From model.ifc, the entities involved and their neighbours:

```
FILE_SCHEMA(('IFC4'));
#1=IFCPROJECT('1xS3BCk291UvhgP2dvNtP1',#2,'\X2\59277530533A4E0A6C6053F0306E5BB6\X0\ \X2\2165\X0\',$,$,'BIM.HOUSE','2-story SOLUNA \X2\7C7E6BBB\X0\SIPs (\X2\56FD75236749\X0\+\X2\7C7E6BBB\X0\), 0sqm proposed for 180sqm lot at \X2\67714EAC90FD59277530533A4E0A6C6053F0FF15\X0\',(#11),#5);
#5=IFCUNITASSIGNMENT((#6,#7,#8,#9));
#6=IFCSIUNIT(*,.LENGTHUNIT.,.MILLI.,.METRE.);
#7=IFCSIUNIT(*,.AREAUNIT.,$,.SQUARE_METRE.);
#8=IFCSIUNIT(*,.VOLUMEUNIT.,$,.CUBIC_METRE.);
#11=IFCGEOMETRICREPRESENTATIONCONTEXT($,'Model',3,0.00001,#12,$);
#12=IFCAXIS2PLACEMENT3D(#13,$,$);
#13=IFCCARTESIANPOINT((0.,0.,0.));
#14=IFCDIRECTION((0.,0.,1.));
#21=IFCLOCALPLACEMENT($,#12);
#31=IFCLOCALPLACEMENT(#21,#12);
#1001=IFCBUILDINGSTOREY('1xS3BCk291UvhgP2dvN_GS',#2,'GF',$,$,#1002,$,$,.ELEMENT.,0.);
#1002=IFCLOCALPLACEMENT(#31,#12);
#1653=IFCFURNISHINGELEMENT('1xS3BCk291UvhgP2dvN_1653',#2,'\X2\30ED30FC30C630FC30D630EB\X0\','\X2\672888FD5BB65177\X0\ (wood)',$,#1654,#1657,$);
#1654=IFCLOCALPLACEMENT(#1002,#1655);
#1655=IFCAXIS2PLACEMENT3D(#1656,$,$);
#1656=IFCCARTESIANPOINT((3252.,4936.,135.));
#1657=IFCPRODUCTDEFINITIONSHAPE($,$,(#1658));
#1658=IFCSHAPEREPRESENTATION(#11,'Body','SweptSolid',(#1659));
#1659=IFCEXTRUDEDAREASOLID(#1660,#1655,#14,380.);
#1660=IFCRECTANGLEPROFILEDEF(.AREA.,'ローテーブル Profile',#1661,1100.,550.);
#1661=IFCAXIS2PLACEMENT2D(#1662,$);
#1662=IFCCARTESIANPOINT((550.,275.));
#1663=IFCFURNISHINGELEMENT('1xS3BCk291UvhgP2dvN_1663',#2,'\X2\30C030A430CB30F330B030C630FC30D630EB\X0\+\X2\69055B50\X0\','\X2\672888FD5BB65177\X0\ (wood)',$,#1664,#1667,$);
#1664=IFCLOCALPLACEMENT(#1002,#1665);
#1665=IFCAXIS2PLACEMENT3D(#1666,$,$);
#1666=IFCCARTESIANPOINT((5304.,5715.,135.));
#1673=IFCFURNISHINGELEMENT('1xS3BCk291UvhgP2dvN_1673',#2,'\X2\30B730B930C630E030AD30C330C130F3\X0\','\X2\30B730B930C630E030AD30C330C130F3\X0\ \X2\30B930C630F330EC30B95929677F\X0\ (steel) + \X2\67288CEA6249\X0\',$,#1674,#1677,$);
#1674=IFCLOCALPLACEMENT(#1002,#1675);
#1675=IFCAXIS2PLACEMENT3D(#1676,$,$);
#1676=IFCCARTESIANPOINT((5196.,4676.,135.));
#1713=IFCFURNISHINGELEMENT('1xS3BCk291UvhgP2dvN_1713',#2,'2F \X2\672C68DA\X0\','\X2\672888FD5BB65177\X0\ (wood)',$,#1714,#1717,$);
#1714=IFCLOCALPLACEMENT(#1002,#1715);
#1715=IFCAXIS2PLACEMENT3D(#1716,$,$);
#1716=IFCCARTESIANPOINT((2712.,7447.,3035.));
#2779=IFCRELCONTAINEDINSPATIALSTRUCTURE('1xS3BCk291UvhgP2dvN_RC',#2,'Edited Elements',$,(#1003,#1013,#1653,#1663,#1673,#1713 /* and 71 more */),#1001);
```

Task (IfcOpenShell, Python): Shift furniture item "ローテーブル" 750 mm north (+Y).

```python
import ifcopenshell
import ifcopenshell.api.geometry
import ifcopenshell.util.placement
import ifcopenshell.util.unit

model = ifcopenshell.open("model.ifc")
unit_scale = ifcopenshell.util.unit.calculate_unit_scale(model)

item = model.by_id(1653)
matrix = ifcopenshell.util.placement.get_local_placement(item.ObjectPlacement)
matrix[1, 3] += 0.75 / unit_scale
ifcopenshell.api.geometry.edit_object_placement(model, product=item, matrix=matrix, is_si=False)

print(ifcopenshell.util.placement.get_local_placement(item.ObjectPlacement).round(3) + 0.0)

model.write("model_edited.ifc")
```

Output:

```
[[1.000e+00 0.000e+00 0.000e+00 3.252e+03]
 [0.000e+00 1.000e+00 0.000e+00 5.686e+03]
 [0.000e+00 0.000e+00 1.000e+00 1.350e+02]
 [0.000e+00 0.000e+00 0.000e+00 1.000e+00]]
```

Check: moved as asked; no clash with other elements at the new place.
